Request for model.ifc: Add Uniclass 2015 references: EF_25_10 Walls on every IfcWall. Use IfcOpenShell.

First a look at what the model holds.

```python
import ifcopenshell

model = ifcopenshell.open("model.ifc")
print(model.schema)
print("classifications:", [c.Name for c in model.by_type("IfcClassification")])
for ifc_class in ("IfcDoor", "IfcRoof", "IfcStair", "IfcWall", "IfcWindow"):
    print(ifc_class, len(model.by_type(ifc_class)))
```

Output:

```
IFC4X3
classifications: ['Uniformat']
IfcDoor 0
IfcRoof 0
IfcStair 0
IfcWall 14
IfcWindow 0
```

```python
import ifcopenshell
import ifcopenshell.api.classification

model = ifcopenshell.open("model.ifc")

system = ifcopenshell.api.classification.add_classification(model, classification="Uniclass 2015")

codes = {
    "IfcWall": ("EF_25_10", "Walls"),
}
for ifc_class, (code, name) in codes.items():
    products = model.by_type(ifc_class)
    ifcopenshell.api.classification.add_reference(
        model, products=products, classification=system, identification=code, name=name
    )
    print(code, len(products))

model.write("model-out.ifc")
```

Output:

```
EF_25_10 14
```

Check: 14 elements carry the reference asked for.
